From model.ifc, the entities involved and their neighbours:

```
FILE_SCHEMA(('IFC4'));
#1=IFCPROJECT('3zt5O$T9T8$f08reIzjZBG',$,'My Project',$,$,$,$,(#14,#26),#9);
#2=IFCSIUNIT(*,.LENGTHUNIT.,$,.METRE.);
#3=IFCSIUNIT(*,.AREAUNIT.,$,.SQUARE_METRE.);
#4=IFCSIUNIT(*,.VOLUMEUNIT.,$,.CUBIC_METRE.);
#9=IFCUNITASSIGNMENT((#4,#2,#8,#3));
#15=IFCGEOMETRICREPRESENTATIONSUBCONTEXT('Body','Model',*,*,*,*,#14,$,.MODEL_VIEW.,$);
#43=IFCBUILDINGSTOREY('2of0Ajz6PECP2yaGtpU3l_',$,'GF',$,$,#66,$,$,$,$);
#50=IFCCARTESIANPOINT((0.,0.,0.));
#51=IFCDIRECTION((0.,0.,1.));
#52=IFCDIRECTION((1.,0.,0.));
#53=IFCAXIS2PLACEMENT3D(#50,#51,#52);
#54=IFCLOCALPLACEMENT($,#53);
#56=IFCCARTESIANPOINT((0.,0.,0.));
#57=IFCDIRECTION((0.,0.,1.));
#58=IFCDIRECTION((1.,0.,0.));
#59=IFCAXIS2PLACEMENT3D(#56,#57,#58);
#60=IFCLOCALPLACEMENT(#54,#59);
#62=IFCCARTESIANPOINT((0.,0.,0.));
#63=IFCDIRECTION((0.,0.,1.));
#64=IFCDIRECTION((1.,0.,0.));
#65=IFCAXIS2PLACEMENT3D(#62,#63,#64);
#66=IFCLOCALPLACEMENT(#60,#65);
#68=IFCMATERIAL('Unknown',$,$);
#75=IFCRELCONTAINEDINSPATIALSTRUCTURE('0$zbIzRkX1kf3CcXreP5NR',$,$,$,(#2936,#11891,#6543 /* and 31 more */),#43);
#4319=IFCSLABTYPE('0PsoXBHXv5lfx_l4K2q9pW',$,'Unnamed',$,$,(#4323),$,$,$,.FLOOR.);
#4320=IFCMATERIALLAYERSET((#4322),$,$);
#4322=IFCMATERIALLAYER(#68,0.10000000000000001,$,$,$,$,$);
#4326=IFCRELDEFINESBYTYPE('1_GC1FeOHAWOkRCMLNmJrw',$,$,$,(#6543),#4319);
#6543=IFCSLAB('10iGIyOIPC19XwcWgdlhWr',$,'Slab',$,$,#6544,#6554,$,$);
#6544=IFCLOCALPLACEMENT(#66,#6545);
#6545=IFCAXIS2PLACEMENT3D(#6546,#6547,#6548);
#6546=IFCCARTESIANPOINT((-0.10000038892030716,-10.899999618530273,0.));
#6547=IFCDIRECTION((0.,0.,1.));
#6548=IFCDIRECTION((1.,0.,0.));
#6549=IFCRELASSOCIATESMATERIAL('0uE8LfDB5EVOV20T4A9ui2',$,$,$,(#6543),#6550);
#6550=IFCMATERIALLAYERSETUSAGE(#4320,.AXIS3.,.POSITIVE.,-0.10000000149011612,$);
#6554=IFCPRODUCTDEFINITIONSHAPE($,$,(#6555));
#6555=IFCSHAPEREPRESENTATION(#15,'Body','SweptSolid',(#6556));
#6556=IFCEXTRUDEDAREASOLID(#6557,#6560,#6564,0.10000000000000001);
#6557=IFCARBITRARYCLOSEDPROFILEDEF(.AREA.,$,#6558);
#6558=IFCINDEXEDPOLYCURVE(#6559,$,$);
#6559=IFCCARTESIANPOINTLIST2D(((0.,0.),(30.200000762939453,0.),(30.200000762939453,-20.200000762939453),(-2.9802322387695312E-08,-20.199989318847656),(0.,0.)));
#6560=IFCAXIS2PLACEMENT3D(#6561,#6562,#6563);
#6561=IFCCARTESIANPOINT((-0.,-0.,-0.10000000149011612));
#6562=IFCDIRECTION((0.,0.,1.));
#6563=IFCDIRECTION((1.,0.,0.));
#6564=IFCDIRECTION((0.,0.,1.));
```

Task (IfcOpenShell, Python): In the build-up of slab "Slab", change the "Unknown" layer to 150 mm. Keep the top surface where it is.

```python
import ifcopenshell
import ifcopenshell.util.element
import ifcopenshell.util.representation
import ifcopenshell.util.unit

model = ifcopenshell.open("model.ifc")
unit_scale = ifcopenshell.util.unit.calculate_unit_scale(model)

layer_set = model.by_id(4320)
layer = next(l for l in layer_set.MaterialLayers if l.Material and l.Material.Name == "Unknown")
change = 0.15 / unit_scale - layer.LayerThickness
layer.LayerThickness += change

# Geometry does not follow the layer set by itself.
slabs = [e for e in ifcopenshell.util.element.get_elements_by_material(model, layer_set) if e.is_a("IfcSlab")]
for slab in sorted(slabs, key=lambda e: e.id()):
    body = ifcopenshell.util.representation.get_representation(slab, "Model", "Body")
    solid = body.Items[0]
    old_depth = solid.Depth
    solid.Depth += change
    # Extruded upwards: lower the start of the extrusion so the top stays.
    x, y, z = solid.Position.Location.Coordinates
    solid.Position.Location = model.createIfcCartesianPoint((x, y, z - change))
    print(slab.id(), f"{old_depth:g} -> {solid.Depth:g}")

# The layers are counted up from the underside, which has moved.
for usage in {ifcopenshell.util.element.get_material(slab) for slab in slabs}:
    usage.OffsetFromReferenceLine -= change

model.write("model_edited.ifc")
```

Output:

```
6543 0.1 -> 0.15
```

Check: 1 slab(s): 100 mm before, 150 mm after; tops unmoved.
